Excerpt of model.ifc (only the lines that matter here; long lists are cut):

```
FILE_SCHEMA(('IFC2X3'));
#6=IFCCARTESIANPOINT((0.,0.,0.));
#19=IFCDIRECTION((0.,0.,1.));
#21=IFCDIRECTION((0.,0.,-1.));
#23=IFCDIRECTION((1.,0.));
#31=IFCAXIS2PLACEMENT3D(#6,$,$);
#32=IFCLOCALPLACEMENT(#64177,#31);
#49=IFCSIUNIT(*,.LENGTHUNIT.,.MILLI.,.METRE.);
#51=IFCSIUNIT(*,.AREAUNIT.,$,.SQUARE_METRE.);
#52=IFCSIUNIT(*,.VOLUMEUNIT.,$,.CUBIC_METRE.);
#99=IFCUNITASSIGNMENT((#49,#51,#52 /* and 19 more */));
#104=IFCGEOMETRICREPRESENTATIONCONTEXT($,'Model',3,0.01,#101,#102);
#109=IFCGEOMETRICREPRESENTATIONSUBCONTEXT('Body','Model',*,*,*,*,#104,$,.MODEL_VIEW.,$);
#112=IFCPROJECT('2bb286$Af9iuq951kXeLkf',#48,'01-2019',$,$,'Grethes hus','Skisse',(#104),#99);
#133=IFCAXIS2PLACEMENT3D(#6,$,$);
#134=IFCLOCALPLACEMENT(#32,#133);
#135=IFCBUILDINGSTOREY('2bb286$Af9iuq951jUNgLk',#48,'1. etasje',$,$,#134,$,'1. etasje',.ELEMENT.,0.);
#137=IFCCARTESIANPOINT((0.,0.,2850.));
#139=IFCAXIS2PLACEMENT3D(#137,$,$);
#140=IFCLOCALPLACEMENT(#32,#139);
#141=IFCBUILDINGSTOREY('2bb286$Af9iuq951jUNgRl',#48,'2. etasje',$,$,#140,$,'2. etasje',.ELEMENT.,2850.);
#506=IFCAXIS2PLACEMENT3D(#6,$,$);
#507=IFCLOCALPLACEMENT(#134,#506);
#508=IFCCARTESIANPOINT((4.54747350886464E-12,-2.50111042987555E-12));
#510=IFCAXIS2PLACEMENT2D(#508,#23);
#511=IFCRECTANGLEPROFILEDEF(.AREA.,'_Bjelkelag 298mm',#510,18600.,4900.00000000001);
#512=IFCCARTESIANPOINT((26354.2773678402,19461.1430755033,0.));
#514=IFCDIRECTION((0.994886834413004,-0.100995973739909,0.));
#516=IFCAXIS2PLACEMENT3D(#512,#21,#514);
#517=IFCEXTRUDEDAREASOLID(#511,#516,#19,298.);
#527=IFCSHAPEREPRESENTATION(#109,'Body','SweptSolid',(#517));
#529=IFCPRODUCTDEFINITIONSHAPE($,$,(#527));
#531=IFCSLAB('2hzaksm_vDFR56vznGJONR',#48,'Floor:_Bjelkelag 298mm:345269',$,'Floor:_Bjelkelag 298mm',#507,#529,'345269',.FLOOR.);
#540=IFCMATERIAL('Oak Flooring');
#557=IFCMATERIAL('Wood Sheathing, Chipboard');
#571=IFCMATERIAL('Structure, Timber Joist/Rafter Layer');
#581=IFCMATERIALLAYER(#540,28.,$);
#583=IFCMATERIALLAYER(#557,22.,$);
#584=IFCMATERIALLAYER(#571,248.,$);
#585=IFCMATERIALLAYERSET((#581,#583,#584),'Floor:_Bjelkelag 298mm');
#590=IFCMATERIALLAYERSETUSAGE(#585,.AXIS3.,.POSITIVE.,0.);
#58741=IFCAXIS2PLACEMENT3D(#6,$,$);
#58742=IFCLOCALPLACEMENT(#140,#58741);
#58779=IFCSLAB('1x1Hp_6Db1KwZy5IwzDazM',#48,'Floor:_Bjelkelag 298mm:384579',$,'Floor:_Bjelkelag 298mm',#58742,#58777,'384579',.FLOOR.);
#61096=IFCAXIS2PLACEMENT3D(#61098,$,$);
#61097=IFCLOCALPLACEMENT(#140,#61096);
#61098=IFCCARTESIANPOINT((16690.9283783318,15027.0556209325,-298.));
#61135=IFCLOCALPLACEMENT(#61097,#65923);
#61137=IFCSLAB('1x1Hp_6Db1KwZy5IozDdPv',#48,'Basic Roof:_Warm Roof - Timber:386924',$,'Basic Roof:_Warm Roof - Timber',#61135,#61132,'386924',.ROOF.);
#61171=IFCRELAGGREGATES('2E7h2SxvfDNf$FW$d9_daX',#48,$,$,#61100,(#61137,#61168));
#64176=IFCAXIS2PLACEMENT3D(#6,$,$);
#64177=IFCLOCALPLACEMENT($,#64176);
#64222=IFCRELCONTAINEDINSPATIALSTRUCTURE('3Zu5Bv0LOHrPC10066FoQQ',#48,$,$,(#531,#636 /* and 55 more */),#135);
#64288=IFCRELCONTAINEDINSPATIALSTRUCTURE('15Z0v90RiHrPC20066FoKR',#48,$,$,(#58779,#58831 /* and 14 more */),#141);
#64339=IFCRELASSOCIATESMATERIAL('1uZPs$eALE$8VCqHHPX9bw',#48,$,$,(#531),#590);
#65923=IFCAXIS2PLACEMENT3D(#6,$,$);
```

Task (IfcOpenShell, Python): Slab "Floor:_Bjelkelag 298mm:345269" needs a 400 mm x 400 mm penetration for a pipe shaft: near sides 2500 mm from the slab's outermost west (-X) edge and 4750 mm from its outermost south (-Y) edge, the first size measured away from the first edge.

```python
import numpy as np
import ifcopenshell
import ifcopenshell.api.feature
import ifcopenshell.api.geometry
import ifcopenshell.api.root
import ifcopenshell.geom
import ifcopenshell.util.placement
import ifcopenshell.util.representation
import ifcopenshell.util.shape
import ifcopenshell.util.unit

model = ifcopenshell.open("model.ifc")
unit_scale = ifcopenshell.util.unit.calculate_unit_scale(model)
settings = ifcopenshell.geom.settings()


def volume(element):
    """Net volume in cubic metres, openings subtracted."""
    shape = ifcopenshell.geom.create_shape(settings, element)
    return ifcopenshell.util.shape.get_volume(shape.geometry)


slab = model.by_id(531)
before = volume(slab)

# Extent in the slab's own axes, in metres. The edges named are its -X and -Y sides.
slab_shape = ifcopenshell.geom.create_shape(settings, slab)
vertices = ifcopenshell.util.shape.get_vertices(slab_shape.geometry)
x_min, y_min, bottom = vertices.min(axis=0)
top = vertices[:, 2].max()

opening = ifcopenshell.api.root.create_entity(model, ifc_class="IfcOpeningElement", name="Pipe shaft opening")
context = ifcopenshell.util.representation.get_context(model, "Model", "Body", "MODEL_VIEW")
width, depth = 0.4, 0.4
outline = [(0.0, 0.0), (width, 0.0), (width, depth), (0.0, depth), (0.0, 0.0)]
# Overshoot both faces by 50 mm so the cut is clean.
shape = ifcopenshell.api.geometry.add_slab_representation(
    model, context=context, depth=top - bottom + 0.1, polyline=outline
)
ifcopenshell.api.geometry.assign_representation(model, product=opening, representation=shape)

matrix = ifcopenshell.util.placement.get_local_placement(slab.ObjectPlacement)
matrix[:, 3] = matrix @ np.append(np.array([x_min + 2.5, y_min + 4.75, bottom - 0.05]) / unit_scale, 1.0)
ifcopenshell.api.geometry.edit_object_placement(model, product=opening, matrix=matrix, is_si=False)
ifcopenshell.api.feature.add_feature(model, feature=opening, element=slab)

after = volume(slab)

print(f"slab volume {before:.3f} -> {after:.3f} m3")

model.write("model_rev.ifc")
```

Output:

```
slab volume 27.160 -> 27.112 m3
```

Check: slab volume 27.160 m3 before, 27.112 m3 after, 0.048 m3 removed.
